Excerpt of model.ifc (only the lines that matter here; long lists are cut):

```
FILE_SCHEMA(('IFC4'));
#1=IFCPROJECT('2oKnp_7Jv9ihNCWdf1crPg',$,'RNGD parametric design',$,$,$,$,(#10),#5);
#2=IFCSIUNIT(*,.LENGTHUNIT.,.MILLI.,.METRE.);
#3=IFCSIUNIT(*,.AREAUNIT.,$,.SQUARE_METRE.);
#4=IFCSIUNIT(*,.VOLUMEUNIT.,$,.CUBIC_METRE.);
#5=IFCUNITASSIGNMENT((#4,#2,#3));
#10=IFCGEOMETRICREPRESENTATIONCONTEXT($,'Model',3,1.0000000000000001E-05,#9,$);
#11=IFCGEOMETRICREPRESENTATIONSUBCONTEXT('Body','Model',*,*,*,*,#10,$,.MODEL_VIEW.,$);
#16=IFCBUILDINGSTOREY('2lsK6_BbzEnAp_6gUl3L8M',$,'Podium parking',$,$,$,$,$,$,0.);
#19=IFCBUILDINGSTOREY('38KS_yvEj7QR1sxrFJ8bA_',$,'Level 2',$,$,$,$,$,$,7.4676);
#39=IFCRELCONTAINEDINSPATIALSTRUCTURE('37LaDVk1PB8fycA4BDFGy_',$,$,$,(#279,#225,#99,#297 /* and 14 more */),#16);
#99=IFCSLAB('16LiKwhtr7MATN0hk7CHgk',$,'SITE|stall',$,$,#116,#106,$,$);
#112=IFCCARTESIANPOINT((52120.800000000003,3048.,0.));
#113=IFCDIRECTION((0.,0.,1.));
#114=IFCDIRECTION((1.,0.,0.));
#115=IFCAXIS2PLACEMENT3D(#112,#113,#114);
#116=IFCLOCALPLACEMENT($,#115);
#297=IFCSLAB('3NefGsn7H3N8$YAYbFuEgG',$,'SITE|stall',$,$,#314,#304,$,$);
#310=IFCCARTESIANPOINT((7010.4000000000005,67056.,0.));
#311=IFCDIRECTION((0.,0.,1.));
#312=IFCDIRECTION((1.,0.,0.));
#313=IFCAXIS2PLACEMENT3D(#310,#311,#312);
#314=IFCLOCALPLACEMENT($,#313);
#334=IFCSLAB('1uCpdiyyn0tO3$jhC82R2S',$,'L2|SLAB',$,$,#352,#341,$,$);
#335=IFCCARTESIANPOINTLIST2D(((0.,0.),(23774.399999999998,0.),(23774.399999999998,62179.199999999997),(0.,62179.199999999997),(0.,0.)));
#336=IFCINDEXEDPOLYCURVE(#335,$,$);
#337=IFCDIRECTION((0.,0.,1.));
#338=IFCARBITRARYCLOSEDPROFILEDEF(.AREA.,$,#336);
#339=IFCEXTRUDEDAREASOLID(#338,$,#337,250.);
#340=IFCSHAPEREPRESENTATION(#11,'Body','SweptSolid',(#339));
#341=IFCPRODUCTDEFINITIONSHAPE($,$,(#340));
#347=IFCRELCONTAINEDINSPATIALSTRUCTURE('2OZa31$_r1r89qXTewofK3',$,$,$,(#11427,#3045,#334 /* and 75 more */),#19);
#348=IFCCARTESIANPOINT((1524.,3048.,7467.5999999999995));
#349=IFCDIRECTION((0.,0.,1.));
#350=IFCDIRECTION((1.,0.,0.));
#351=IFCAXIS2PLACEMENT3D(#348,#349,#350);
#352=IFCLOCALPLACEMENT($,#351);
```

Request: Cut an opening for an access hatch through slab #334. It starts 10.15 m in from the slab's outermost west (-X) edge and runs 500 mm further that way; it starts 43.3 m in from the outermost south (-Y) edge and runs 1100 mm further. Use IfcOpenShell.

```python
import numpy as np
import ifcopenshell
import ifcopenshell.api.feature
import ifcopenshell.api.geometry
import ifcopenshell.api.root
import ifcopenshell.geom
import ifcopenshell.util.placement
import ifcopenshell.util.representation
import ifcopenshell.util.shape
import ifcopenshell.util.unit

model = ifcopenshell.open("model.ifc")
unit_scale = ifcopenshell.util.unit.calculate_unit_scale(model)
settings = ifcopenshell.geom.settings()


def volume(element):
    """Net volume in cubic metres, openings subtracted."""
    shape = ifcopenshell.geom.create_shape(settings, element)
    return ifcopenshell.util.shape.get_volume(shape.geometry)


slab = model.by_id(334)
before = volume(slab)

# Extent in the slab's own axes, in metres. The edges named are its -X and -Y sides.
slab_shape = ifcopenshell.geom.create_shape(settings, slab)
vertices = ifcopenshell.util.shape.get_vertices(slab_shape.geometry)
x_min, y_min, bottom = vertices.min(axis=0)
top = vertices[:, 2].max()

opening = ifcopenshell.api.root.create_entity(model, ifc_class="IfcOpeningElement", name="Access hatch opening", predefined_type="OPENING")
context = ifcopenshell.util.representation.get_context(model, "Model", "Body", "MODEL_VIEW")
width, depth = 0.5, 1.1
outline = [(0.0, 0.0), (width, 0.0), (width, depth), (0.0, depth), (0.0, 0.0)]
# Overshoot both faces by 50 mm so the cut is clean.
shape = ifcopenshell.api.geometry.add_slab_representation(
    model, context=context, depth=top - bottom + 0.1, polyline=outline
)
ifcopenshell.api.geometry.assign_representation(model, product=opening, representation=shape)

matrix = ifcopenshell.util.placement.get_local_placement(slab.ObjectPlacement)
matrix[:, 3] = matrix @ np.append(np.array([x_min + 10.15, y_min + 43.3, bottom - 0.05]) / unit_scale, 1.0)
ifcopenshell.api.geometry.edit_object_placement(model, product=opening, matrix=matrix, is_si=False)
ifcopenshell.api.feature.add_feature(model, feature=opening, element=slab)

after = volume(slab)

print(f"slab volume {before:.3f} -> {after:.3f} m3")

model.write("model_v2.ifc")
```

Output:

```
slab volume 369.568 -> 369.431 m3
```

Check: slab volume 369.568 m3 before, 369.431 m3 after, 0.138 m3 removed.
